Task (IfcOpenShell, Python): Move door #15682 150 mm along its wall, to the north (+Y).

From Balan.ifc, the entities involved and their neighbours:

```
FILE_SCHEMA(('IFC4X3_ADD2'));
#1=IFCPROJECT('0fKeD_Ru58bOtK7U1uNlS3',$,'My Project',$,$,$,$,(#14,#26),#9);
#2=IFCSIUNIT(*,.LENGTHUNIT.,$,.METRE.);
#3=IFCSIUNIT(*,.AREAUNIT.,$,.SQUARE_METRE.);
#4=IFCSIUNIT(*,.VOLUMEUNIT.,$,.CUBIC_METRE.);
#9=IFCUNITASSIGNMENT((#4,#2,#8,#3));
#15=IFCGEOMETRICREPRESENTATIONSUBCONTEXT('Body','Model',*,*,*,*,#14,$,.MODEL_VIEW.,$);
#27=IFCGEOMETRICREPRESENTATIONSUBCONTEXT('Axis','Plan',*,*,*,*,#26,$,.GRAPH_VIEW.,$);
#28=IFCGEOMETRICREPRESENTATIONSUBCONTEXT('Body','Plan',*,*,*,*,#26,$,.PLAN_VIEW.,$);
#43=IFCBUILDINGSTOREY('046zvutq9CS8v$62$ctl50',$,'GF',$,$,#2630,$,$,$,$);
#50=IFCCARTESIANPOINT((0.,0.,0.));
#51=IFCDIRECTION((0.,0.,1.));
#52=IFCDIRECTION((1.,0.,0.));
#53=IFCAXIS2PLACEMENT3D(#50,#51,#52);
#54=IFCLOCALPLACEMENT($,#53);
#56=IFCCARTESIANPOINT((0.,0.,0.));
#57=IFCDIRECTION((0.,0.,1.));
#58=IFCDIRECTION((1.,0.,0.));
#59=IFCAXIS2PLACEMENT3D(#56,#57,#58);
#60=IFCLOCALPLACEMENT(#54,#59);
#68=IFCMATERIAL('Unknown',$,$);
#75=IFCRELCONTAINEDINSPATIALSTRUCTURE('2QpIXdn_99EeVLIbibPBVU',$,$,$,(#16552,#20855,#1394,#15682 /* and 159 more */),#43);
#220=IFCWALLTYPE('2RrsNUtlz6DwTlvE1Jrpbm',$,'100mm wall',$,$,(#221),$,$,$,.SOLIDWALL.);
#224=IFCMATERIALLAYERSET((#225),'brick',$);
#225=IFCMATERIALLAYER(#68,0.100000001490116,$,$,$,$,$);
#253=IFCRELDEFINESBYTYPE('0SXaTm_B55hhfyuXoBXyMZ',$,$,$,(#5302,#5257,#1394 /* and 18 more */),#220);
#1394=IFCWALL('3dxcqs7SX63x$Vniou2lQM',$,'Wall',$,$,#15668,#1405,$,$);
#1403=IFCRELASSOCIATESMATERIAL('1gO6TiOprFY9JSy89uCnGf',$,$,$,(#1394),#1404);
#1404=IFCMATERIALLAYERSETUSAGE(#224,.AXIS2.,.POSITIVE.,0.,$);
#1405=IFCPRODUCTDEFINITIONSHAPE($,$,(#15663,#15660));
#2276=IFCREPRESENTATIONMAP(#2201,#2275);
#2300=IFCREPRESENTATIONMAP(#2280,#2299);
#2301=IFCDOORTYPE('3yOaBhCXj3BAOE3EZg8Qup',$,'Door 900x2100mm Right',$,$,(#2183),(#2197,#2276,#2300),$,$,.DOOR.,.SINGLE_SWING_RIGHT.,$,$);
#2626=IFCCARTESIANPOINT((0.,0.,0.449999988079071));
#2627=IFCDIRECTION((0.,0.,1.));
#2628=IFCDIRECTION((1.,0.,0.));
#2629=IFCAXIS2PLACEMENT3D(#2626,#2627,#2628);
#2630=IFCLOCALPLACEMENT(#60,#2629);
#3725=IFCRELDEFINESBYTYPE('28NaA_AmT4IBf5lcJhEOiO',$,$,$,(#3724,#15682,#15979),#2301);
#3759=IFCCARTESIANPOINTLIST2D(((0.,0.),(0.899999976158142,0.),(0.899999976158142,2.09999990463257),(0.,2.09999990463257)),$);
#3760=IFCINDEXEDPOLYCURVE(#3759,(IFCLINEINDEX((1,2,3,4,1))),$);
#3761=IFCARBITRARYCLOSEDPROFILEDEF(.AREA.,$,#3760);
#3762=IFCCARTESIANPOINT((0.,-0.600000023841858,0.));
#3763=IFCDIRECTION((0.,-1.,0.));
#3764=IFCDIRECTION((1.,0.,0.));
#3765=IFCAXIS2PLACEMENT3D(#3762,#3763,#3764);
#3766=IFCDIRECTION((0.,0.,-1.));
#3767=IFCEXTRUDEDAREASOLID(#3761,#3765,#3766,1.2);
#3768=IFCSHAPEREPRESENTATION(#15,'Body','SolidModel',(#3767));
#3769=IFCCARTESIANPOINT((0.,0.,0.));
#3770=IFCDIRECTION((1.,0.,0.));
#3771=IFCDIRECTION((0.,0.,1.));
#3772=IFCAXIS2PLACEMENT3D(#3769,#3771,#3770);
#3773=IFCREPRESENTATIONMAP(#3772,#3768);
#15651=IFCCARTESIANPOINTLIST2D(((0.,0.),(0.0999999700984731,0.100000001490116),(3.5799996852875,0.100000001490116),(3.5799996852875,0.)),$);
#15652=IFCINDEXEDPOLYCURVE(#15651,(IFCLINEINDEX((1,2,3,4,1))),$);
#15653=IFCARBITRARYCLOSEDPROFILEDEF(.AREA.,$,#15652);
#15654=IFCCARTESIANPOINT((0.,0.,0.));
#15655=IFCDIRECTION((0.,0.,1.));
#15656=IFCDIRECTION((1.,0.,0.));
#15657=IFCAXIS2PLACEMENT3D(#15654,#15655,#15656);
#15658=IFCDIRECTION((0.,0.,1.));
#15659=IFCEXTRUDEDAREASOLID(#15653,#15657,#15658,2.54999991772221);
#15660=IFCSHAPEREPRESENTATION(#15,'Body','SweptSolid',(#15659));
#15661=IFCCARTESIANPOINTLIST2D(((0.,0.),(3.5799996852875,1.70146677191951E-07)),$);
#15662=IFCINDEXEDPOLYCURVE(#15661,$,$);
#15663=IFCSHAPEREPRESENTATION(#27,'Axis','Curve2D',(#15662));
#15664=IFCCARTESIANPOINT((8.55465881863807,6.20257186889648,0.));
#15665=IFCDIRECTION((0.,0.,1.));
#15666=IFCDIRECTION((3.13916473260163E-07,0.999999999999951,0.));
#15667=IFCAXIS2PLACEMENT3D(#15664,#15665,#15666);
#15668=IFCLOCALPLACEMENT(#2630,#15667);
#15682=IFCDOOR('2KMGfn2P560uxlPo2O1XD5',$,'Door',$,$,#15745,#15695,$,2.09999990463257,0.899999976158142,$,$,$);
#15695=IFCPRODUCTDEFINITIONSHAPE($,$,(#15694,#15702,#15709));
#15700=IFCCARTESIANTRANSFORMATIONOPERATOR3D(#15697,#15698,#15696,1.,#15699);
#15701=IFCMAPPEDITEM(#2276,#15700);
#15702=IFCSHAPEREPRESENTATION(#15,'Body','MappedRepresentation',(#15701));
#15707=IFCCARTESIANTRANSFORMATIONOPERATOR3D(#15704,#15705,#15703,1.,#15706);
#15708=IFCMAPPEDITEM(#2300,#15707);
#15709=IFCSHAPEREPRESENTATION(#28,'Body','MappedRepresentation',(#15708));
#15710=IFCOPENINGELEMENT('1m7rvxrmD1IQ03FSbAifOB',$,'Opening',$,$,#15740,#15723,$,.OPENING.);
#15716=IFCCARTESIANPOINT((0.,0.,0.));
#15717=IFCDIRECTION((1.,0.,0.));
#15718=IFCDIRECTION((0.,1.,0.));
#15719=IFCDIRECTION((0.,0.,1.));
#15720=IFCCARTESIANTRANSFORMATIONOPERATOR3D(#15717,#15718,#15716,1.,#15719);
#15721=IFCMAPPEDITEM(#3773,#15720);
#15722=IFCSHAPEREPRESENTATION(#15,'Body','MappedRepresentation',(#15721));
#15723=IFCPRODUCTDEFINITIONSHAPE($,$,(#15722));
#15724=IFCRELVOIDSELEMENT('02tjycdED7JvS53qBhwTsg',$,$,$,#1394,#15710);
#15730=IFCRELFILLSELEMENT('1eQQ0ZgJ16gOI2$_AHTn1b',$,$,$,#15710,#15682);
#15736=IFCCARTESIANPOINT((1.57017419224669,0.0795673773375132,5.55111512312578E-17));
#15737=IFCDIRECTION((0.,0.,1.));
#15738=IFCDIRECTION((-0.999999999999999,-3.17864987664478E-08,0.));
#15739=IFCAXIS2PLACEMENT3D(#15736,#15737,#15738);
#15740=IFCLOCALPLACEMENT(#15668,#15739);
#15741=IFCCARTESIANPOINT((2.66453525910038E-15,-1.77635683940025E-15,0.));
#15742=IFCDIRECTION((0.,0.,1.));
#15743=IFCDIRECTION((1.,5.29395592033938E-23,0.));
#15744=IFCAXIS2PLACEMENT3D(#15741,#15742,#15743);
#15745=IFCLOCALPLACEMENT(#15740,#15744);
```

```python
import ifcopenshell
import ifcopenshell.api.geometry
import ifcopenshell.util.placement
import ifcopenshell.util.unit

model = ifcopenshell.open("Balan.ifc")
unit_scale = ifcopenshell.util.unit.calculate_unit_scale(model)

door = model.by_id(15682)
opening = door.FillsVoids[0].RelatingOpeningElement
wall = opening.VoidsElements[0].RelatingBuildingElement

wall_matrix = ifcopenshell.util.placement.get_local_placement(wall.ObjectPlacement)
shift = wall_matrix[:3, 0] * 0.15 / unit_scale
before = ifcopenshell.util.placement.get_local_placement(door.ObjectPlacement)[:3, 3].copy()

# The door is placed relative to its opening, so it follows when the opening moves.
matrix = ifcopenshell.util.placement.get_local_placement(opening.ObjectPlacement)
matrix[:3, 3] += shift
ifcopenshell.api.geometry.edit_object_placement(
    model, product=opening, matrix=matrix, is_si=False, should_transform_children=True
)

after = ifcopenshell.util.placement.get_local_placement(door.ObjectPlacement)[:3, 3]
print("door moved by", (after - before).round(3) + 0.0)

model.write("Balan-out.ifc")
```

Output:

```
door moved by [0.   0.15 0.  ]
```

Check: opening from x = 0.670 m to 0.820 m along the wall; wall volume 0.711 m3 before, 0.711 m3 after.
